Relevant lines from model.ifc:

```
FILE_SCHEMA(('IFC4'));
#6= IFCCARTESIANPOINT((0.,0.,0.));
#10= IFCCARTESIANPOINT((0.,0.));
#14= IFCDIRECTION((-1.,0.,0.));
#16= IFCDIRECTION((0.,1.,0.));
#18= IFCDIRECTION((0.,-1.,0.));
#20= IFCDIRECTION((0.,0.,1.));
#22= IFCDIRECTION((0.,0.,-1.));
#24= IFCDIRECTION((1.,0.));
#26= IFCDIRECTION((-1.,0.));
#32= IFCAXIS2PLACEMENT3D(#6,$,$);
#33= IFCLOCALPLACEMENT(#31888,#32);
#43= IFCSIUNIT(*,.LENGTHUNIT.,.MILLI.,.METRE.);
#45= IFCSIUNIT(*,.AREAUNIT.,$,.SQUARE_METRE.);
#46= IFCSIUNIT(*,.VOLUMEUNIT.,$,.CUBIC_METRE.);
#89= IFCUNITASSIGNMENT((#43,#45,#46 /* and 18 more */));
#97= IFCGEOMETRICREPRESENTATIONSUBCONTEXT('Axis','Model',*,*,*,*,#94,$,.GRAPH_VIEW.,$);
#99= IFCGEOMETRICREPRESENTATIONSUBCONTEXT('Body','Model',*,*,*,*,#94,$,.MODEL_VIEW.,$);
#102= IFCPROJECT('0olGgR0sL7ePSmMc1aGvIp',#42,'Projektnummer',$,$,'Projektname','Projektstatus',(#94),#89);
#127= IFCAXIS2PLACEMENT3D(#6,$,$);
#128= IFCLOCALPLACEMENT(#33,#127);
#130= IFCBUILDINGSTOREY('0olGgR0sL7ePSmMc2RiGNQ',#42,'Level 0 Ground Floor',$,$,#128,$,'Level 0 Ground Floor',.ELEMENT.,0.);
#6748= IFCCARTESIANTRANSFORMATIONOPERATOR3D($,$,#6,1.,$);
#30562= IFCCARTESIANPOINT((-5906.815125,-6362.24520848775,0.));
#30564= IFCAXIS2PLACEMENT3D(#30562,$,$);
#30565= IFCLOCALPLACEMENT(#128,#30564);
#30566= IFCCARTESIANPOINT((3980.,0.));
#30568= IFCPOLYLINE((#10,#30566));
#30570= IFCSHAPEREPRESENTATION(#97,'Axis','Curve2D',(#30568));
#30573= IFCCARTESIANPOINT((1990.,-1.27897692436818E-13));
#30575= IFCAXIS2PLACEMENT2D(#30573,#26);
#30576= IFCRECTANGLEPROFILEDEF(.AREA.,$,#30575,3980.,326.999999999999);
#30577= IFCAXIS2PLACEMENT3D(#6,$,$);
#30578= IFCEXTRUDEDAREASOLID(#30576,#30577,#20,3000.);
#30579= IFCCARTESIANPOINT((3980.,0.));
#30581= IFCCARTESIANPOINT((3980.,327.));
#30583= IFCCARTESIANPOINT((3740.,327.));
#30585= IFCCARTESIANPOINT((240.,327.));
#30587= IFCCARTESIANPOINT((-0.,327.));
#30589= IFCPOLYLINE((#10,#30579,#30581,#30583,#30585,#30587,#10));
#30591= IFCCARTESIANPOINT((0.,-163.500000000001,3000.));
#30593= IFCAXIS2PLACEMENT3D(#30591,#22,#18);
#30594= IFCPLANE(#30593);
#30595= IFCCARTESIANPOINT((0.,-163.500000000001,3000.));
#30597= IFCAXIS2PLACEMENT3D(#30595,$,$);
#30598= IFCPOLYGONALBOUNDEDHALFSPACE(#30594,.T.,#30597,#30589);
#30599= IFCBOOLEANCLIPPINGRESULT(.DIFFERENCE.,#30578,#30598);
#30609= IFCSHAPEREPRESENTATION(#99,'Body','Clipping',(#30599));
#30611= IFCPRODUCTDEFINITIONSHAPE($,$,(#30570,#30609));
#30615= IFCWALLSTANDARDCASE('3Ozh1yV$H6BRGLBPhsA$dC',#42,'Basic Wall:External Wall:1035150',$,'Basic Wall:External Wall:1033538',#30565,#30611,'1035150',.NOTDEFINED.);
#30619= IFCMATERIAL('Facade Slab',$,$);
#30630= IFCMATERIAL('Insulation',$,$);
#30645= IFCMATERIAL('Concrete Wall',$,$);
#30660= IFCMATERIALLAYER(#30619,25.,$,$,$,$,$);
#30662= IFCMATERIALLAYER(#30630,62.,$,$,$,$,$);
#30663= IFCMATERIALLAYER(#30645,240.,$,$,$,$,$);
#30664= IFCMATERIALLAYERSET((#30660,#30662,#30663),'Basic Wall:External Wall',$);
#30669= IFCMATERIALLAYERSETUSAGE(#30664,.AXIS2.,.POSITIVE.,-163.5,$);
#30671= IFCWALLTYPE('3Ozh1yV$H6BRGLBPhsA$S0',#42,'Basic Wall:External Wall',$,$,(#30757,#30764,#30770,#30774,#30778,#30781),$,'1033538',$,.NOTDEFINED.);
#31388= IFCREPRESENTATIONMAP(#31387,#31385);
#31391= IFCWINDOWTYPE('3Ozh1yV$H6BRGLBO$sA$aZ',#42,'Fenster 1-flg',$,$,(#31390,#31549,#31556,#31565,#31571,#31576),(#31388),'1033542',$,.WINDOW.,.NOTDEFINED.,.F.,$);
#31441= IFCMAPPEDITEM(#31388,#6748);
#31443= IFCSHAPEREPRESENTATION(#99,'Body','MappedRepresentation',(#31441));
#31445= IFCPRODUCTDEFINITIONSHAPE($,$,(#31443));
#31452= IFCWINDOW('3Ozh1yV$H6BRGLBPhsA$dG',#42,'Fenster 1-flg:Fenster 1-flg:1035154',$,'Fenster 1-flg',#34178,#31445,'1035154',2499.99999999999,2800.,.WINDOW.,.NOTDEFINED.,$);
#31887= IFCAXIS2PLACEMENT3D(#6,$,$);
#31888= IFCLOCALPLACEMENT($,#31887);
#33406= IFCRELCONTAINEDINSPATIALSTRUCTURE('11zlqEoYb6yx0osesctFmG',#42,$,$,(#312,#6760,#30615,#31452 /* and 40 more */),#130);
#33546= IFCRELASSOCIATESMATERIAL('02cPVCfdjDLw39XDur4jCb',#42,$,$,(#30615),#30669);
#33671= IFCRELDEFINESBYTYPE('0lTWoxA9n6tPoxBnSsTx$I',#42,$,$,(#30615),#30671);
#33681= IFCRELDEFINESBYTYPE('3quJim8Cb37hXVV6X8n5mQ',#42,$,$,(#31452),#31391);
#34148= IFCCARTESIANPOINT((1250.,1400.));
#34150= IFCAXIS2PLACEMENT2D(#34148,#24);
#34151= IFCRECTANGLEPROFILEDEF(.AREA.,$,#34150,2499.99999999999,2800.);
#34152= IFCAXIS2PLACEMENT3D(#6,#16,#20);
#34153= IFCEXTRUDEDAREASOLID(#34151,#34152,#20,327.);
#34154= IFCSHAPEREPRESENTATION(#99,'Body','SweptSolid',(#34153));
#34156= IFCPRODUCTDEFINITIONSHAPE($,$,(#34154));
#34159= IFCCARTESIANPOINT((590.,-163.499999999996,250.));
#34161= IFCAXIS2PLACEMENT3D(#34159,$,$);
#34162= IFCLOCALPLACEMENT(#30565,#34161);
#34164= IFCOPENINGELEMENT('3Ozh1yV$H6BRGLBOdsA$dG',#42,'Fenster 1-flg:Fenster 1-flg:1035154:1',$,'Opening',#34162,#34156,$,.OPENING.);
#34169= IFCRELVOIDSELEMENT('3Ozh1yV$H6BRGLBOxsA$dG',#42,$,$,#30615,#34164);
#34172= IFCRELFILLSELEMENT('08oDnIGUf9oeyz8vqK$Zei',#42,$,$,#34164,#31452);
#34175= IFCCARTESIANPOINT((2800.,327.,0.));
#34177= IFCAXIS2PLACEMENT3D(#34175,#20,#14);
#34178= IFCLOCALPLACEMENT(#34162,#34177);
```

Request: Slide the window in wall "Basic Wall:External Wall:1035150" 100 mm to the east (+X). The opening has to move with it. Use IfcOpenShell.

```python
import ifcopenshell
import ifcopenshell.api.geometry
import ifcopenshell.util.placement
import ifcopenshell.util.unit

model = ifcopenshell.open("model.ifc")
unit_scale = ifcopenshell.util.unit.calculate_unit_scale(model)

window = model.by_guid("3Ozh1yV$H6BRGLBPhsA$dG")
opening = window.FillsVoids[0].RelatingOpeningElement
wall = opening.VoidsElements[0].RelatingBuildingElement

wall_matrix = ifcopenshell.util.placement.get_local_placement(wall.ObjectPlacement)
shift = wall_matrix[:3, 0] * 0.1 / unit_scale
before = ifcopenshell.util.placement.get_local_placement(window.ObjectPlacement)[:3, 3].copy()

# The window is placed relative to its opening, so it follows when the opening moves.
matrix = ifcopenshell.util.placement.get_local_placement(opening.ObjectPlacement)
matrix[:3, 3] += shift
ifcopenshell.api.geometry.edit_object_placement(
    model, product=opening, matrix=matrix, is_si=False, should_transform_children=True
)

after = ifcopenshell.util.placement.get_local_placement(window.ObjectPlacement)[:3, 3]
print("window moved by", (after - before).round(3) + 0.0)

model.write("model_v2.ifc")
```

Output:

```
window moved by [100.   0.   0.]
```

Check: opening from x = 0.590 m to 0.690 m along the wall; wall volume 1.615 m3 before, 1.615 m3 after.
